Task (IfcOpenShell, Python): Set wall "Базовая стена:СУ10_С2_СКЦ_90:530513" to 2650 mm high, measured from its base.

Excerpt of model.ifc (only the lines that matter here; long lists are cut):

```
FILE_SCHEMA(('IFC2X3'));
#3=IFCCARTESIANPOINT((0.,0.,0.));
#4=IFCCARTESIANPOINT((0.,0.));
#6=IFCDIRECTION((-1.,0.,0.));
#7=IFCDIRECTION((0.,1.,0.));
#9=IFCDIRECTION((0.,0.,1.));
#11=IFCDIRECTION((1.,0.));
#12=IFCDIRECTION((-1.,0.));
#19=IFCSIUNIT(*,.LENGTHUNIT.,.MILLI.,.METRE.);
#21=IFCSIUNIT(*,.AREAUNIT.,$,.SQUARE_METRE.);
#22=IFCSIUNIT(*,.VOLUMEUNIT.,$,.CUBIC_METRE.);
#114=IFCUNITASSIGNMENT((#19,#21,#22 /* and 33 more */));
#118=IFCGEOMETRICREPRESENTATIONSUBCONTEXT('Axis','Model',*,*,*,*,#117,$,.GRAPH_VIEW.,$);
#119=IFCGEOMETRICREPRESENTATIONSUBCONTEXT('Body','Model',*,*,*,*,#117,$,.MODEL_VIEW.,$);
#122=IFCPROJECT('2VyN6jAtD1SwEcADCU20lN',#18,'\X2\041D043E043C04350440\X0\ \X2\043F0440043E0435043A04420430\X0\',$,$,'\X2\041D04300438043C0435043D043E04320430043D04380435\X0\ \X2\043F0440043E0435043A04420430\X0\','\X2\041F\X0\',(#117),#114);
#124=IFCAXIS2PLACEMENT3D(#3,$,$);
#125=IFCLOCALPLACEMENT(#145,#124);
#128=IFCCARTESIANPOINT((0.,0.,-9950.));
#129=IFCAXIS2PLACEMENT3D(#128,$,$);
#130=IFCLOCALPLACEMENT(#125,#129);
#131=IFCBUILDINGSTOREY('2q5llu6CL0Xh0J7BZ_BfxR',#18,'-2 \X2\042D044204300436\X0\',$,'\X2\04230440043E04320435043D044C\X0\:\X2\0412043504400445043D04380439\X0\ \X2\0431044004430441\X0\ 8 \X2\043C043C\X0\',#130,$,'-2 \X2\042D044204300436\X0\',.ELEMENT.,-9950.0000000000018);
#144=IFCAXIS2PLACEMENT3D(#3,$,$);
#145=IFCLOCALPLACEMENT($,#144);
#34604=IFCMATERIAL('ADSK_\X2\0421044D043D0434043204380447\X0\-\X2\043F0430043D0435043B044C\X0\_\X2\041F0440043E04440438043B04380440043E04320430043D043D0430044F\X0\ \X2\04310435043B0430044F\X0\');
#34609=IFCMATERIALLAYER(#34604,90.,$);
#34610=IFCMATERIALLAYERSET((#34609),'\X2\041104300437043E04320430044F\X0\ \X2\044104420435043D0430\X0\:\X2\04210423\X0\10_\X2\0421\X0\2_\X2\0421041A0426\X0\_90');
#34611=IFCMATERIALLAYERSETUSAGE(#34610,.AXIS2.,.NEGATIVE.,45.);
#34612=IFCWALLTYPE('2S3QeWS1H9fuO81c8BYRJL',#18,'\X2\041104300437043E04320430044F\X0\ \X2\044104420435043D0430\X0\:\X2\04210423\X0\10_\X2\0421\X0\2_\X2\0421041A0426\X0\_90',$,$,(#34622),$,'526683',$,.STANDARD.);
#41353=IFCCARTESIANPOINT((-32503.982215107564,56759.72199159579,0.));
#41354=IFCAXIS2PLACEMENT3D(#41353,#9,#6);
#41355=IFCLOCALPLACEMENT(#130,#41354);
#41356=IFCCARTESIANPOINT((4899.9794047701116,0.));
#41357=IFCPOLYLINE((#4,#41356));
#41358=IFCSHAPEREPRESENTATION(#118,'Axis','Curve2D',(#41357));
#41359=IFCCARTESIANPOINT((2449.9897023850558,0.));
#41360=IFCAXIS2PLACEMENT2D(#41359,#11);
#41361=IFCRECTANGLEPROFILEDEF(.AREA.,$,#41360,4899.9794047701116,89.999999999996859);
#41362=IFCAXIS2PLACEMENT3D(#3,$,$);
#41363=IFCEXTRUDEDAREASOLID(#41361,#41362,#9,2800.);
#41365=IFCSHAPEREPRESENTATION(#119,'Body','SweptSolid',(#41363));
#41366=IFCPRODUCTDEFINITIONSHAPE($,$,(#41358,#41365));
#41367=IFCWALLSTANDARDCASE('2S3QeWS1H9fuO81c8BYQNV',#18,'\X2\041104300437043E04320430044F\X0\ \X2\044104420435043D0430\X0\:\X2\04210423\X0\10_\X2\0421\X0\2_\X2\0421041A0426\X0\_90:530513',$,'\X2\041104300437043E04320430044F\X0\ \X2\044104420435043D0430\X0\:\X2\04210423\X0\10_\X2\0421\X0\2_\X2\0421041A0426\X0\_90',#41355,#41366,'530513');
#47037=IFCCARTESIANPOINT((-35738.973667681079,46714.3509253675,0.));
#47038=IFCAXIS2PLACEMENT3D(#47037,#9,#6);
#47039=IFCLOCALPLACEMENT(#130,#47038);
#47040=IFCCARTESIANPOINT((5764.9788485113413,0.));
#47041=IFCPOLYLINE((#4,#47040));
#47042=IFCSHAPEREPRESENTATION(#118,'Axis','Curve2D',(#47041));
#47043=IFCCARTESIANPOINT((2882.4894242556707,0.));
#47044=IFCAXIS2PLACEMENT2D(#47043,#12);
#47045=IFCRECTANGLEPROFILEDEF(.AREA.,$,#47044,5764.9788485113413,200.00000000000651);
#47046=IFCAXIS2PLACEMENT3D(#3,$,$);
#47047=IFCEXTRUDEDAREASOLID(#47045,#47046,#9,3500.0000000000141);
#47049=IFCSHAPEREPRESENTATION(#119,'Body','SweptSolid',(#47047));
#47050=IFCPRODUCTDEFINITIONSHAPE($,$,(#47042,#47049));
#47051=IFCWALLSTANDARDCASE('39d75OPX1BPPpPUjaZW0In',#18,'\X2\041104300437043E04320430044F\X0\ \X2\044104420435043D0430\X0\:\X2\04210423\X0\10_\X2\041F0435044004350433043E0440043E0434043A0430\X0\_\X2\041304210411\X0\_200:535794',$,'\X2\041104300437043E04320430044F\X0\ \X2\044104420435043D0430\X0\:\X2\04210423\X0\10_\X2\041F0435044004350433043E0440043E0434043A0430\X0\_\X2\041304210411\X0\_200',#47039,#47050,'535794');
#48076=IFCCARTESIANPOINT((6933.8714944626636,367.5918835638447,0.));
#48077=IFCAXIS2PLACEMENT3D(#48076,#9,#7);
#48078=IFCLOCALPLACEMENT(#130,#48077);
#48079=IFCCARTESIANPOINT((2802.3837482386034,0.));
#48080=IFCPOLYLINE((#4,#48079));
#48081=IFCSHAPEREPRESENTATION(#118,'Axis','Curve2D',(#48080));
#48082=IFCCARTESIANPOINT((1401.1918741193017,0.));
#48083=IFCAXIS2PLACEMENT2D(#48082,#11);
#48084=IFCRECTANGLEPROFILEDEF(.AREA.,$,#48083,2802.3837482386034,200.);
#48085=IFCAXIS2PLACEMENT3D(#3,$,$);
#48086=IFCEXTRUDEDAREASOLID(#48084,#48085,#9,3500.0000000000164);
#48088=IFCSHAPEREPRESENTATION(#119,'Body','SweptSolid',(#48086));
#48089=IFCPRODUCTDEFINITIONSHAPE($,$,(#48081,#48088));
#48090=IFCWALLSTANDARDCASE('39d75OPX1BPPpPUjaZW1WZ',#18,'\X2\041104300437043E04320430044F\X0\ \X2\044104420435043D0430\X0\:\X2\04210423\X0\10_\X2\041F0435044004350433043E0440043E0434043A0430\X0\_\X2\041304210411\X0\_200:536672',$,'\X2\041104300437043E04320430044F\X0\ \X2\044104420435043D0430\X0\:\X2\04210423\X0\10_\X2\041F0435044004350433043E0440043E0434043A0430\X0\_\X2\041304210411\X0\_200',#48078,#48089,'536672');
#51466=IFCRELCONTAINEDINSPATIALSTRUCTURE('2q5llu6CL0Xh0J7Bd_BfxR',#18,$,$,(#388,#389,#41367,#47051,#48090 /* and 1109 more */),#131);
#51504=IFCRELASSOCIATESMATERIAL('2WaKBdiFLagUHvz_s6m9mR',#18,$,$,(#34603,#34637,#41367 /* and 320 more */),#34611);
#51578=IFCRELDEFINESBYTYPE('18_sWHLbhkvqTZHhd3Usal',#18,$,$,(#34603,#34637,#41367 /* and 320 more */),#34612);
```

```python
import ifcopenshell
import ifcopenshell.geom
import ifcopenshell.util.representation
import ifcopenshell.util.shape
import ifcopenshell.util.unit

model = ifcopenshell.open("model.ifc")
unit_scale = ifcopenshell.util.unit.calculate_unit_scale(model)
settings = ifcopenshell.geom.settings()


def volume(element):
    """Net volume in cubic metres, openings subtracted."""
    shape = ifcopenshell.geom.create_shape(settings, element)
    return ifcopenshell.util.shape.get_volume(shape.geometry)


wall = model.by_guid("2S3QeWS1H9fuO81c8BYQNV")
before = volume(wall)

body = ifcopenshell.util.representation.get_representation(wall, "Model", "Body")
solid = body.Items[0]
old_height = solid.Depth
solid.Depth = 2.65 / unit_scale
after = volume(wall)

print(f"height {old_height:g} -> {solid.Depth:g}, volume {before:.3f} -> {after:.3f} m3")

model.write("model_rev.ifc")
```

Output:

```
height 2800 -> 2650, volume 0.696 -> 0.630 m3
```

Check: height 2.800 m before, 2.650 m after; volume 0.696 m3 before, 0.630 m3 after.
